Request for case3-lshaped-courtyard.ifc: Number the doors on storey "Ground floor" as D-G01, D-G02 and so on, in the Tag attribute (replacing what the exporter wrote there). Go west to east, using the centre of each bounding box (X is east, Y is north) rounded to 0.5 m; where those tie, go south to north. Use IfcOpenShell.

First a look at what the model holds.

```python
import ifcopenshell
import ifcopenshell.util.element
import ifcopenshell.util.placement

model = ifcopenshell.open("case3-lshaped-courtyard.ifc")
print(model.schema)
storey = next(s for s in model.by_type("IfcBuildingStorey") if s.Name == "Ground floor")
doors = [e for e in ifcopenshell.util.element.get_decomposition(storey) if e.is_a("IfcDoor")]
for e in sorted(doors, key=lambda e: e.id()):
    origin = ifcopenshell.util.placement.get_local_placement(e.ObjectPlacement)[:3, 3]
    print(e.id(), e.Tag, e.Name, origin.round(2) + 0.0, sep=" | ")
```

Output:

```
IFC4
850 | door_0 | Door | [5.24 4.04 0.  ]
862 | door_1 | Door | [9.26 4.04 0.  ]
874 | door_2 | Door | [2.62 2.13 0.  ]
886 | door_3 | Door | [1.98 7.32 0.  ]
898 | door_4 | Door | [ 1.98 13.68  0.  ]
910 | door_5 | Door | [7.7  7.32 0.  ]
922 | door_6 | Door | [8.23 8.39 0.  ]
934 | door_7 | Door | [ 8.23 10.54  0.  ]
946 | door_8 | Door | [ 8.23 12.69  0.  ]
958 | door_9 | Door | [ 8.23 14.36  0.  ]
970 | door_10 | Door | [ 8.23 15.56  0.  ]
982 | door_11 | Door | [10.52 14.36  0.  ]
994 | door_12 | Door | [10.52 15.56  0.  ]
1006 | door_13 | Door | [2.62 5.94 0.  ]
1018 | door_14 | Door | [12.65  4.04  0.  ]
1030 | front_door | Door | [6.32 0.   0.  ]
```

```python
import ifcopenshell
import ifcopenshell.geom
import ifcopenshell.util.element
import ifcopenshell.util.shape

model = ifcopenshell.open("case3-lshaped-courtyard.ifc")
settings = ifcopenshell.geom.settings()
settings.set("use-world-coords", True)


def centre(element):
    shape = ifcopenshell.geom.create_shape(settings, element)
    return ifcopenshell.util.shape.get_bbox_centroid(shape.geometry)


storey = next(s for s in model.by_type("IfcBuildingStorey") if s.Name == "Ground floor")
doors = [e for e in ifcopenshell.util.element.get_decomposition(storey) if e.is_a("IfcDoor")]

# Insertion points can sit at a corner or the storey origin, so sort by the geometry (in metres).
centres = {e: centre(e) for e in doors}
doors.sort(key=lambda e: (round(centres[e][0] / 0.5), centres[e][1]))

for i, e in enumerate(doors, start=1):
    number = f"D-G{i:02d}"
    e.Tag = number
    print(e.id(), number)

model.write("case3-lshaped-courtyard_updated.ifc")
```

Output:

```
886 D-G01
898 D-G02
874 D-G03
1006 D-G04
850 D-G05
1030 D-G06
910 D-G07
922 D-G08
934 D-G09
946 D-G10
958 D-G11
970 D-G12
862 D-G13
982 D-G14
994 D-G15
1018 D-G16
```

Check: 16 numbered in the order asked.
